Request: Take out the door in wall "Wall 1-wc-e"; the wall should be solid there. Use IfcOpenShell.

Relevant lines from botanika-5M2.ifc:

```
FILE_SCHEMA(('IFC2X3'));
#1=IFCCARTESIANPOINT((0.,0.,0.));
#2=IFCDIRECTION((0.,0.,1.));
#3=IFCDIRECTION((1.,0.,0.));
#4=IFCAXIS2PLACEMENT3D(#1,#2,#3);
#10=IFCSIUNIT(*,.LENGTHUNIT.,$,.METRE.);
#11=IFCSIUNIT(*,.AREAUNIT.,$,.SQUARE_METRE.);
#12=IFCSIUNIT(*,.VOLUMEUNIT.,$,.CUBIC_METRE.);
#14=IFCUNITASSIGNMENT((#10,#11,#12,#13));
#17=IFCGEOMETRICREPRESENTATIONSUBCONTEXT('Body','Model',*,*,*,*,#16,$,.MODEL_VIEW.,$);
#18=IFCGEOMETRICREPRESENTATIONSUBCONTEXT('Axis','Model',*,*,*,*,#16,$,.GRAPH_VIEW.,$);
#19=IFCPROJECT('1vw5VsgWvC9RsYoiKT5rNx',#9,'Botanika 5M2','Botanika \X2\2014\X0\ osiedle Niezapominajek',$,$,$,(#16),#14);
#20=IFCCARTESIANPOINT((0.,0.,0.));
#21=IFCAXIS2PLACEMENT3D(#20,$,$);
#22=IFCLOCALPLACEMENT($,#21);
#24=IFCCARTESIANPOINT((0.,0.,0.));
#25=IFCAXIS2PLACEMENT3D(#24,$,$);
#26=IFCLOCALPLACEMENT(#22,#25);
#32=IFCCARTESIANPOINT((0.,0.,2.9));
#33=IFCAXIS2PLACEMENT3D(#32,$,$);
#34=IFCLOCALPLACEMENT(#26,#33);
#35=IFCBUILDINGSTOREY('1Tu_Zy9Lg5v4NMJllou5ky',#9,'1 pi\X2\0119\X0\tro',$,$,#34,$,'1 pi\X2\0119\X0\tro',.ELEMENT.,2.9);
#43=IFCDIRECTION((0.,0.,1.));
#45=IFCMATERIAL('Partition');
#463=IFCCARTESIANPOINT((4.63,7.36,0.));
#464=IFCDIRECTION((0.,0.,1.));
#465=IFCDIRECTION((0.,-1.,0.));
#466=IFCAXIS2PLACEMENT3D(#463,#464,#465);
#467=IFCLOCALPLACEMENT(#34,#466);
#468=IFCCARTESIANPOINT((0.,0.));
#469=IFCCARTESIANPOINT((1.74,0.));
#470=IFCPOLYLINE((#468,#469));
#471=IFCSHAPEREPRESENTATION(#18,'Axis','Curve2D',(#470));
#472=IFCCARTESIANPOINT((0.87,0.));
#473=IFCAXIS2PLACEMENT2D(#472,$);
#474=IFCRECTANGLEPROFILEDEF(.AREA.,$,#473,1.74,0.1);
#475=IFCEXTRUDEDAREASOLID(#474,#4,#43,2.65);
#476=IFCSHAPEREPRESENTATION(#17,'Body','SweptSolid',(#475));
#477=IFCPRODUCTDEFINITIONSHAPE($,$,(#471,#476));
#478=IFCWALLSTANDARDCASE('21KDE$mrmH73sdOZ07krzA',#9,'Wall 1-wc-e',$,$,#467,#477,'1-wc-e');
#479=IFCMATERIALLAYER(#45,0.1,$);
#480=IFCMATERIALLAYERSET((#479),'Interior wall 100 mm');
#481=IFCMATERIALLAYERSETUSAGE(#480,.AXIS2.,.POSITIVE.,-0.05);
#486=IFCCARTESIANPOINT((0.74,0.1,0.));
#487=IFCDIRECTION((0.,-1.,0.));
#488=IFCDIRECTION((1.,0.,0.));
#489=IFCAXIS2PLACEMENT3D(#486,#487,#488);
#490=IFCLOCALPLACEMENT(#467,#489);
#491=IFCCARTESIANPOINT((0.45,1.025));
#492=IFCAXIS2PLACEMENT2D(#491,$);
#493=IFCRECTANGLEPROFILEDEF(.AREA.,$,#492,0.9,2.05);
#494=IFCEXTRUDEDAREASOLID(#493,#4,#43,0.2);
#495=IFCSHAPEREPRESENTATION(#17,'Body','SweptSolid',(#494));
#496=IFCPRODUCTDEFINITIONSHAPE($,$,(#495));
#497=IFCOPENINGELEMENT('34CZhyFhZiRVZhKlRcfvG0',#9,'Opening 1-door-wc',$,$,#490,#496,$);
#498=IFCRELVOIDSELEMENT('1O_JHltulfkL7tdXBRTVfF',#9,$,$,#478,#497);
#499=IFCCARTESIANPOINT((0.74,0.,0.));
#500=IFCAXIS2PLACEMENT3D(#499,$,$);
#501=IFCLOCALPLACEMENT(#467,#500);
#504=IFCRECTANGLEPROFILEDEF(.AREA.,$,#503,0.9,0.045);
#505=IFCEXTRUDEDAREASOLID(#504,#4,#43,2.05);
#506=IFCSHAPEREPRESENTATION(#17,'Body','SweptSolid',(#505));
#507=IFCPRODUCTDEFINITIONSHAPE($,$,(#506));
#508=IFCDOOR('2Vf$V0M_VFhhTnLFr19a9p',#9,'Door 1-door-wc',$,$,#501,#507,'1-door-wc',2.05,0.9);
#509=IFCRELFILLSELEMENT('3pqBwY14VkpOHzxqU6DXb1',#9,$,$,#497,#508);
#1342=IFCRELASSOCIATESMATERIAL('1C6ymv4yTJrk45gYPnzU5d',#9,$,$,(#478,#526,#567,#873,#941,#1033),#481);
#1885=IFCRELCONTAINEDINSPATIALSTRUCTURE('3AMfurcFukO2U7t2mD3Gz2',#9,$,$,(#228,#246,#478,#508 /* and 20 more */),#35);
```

```python
import ifcopenshell
import ifcopenshell.api.feature
import ifcopenshell.api.root
import ifcopenshell.geom
import ifcopenshell.util.shape

model = ifcopenshell.open("botanika-5M2.ifc")
settings = ifcopenshell.geom.settings()


def volume(element):
    """Net volume in cubic metres, openings subtracted."""
    shape = ifcopenshell.geom.create_shape(settings, element)
    return ifcopenshell.util.shape.get_volume(shape.geometry)


door = model.by_guid("2Vf$V0M_VFhhTnLFr19a9p")
opening = door.FillsVoids[0].RelatingOpeningElement
wall = opening.VoidsElements[0].RelatingBuildingElement
before = volume(wall)

ifcopenshell.api.root.remove_product(model, product=door)
ifcopenshell.api.feature.remove_feature(model, feature=opening)

after = volume(wall)

print(f"wall volume {before:.3f} -> {after:.3f} m3")

model.write("botanika-5M2_updated.ifc")
```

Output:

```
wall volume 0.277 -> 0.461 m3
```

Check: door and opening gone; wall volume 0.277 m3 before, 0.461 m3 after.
